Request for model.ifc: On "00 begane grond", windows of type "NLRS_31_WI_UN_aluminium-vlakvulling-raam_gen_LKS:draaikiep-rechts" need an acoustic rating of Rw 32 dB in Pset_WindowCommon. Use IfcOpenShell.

First a look at what the model holds.

```python
import ifcopenshell
import ifcopenshell.util.element

model = ifcopenshell.open("model.ifc")
print(model.schema)
storey = next(s for s in model.by_type("IfcBuildingStorey") if s.Name == "00 begane grond")
windows = [e for e in ifcopenshell.util.element.get_decomposition(storey) if e.is_a("IfcWindow")]
seen = {}
for e in windows:
    element_type = ifcopenshell.util.element.get_type(e)
    key = (element_type.Name if element_type != e and element_type else None, ifcopenshell.util.element.get_pset(e, "Pset_WindowCommon", "AcousticRating"))
    seen[key] = seen.get(key, 0) + 1
for (name, value), count in sorted(seen.items(), key=str):
    print(count, "x", name, "|", value)
```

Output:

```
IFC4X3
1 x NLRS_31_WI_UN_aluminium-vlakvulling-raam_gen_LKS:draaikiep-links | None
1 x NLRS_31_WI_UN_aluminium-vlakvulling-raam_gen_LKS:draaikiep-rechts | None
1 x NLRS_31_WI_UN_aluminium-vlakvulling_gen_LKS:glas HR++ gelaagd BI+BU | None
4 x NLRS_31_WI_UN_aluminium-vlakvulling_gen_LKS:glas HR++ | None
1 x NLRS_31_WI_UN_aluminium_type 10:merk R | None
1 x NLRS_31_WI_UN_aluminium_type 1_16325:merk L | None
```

```python
import ifcopenshell
import ifcopenshell.api.pset
import ifcopenshell.util.element

model = ifcopenshell.open("model.ifc")

storey = next(s for s in model.by_type("IfcBuildingStorey") if s.Name == "00 begane grond")
windows = [e for e in ifcopenshell.util.element.get_decomposition(storey) if e.is_a("IfcWindow")]

count = 0
for e in windows:
    element_type = ifcopenshell.util.element.get_type(e)
    if element_type in (None, e) or element_type.Name != "NLRS_31_WI_UN_aluminium-vlakvulling-raam_gen_LKS:draaikiep-rechts":
        continue
    # add_pset returns the element's existing set when there is one.
    pset = ifcopenshell.api.pset.add_pset(model, product=e, name="Pset_WindowCommon")
    ifcopenshell.api.pset.edit_pset(model, pset=pset, properties={"AcousticRating": "Rw 32 dB"})
    count += 1

print(count, "windows updated")

model.write("model_updated.ifc")
```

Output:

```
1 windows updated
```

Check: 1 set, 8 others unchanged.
